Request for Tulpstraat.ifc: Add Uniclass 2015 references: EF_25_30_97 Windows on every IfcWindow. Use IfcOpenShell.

First a look at what the model holds.

```python
import ifcopenshell

model = ifcopenshell.open("Tulpstraat.ifc")
print(model.schema)
print("classifications:", [c.Name for c in model.by_type("IfcClassification")])
for ifc_class in ("IfcDoor", "IfcRoof", "IfcStair", "IfcWall", "IfcWindow"):
    print(ifc_class, len(model.by_type(ifc_class)))
```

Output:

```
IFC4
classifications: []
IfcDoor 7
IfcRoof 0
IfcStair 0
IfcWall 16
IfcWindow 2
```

```python
import ifcopenshell
import ifcopenshell.api.classification

model = ifcopenshell.open("Tulpstraat.ifc")

system = ifcopenshell.api.classification.add_classification(model, classification="Uniclass 2015")

codes = {
    "IfcWindow": ("EF_25_30_97", "Windows"),
}
for ifc_class, (code, name) in codes.items():
    products = model.by_type(ifc_class)
    ifcopenshell.api.classification.add_reference(
        model, products=products, classification=system, identification=code, name=name
    )
    print(code, len(products))

model.write("Tulpstraat-out.ifc")
```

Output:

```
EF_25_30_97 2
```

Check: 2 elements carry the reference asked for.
